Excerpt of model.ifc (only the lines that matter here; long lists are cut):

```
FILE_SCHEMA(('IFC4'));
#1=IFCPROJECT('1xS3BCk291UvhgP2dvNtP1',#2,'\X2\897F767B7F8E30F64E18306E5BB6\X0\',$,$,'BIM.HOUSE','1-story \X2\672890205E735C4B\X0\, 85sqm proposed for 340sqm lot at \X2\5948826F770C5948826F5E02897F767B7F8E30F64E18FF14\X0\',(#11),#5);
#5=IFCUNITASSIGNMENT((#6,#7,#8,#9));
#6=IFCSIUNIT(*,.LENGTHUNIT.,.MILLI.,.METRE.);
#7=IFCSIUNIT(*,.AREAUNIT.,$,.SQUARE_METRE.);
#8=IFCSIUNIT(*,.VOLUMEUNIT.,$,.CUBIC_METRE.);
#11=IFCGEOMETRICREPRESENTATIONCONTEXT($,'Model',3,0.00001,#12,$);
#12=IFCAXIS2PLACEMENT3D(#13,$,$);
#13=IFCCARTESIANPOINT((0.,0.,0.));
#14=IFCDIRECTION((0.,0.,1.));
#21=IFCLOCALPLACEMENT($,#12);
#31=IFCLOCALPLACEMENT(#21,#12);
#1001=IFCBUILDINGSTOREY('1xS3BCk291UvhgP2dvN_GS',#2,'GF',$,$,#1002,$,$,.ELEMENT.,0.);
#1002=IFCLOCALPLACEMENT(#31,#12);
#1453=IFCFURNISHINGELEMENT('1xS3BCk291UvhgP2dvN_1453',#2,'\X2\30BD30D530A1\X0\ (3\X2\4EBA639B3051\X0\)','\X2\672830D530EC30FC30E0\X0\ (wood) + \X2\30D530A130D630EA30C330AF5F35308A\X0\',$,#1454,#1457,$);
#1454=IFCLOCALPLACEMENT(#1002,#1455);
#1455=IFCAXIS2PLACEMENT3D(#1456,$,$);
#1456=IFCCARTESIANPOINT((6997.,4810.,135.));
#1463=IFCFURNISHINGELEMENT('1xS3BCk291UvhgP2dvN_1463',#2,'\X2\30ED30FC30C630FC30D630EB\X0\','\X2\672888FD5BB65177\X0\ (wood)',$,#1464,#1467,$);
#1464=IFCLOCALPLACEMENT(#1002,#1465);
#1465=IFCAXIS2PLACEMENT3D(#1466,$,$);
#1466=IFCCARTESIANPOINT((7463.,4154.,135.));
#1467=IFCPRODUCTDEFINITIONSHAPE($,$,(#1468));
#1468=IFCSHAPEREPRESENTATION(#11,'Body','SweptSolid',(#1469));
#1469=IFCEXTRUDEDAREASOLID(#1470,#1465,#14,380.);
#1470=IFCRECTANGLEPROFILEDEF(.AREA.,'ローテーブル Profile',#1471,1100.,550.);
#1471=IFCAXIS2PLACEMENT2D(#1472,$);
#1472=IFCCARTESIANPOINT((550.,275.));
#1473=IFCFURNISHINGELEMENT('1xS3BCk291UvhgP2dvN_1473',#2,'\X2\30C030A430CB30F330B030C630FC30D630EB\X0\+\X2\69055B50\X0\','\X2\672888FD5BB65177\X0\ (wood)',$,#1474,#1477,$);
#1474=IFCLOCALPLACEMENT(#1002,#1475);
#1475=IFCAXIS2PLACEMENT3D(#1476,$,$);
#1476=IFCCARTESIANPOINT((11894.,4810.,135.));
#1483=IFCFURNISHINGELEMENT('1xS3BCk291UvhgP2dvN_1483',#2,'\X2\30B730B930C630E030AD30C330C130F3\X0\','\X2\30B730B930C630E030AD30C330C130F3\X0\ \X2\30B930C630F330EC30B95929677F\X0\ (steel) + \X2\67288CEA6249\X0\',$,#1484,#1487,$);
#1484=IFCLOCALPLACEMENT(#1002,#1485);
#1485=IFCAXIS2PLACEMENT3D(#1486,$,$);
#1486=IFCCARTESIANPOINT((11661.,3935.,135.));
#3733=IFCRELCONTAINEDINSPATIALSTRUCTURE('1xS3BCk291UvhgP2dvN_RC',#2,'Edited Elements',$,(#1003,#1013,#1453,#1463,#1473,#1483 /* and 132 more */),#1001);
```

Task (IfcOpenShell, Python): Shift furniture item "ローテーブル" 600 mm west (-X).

```python
import ifcopenshell
import ifcopenshell.api.geometry
import ifcopenshell.util.placement

model = ifcopenshell.open("model.ifc")

item = model.by_id(1463)
matrix = ifcopenshell.util.placement.get_local_placement(item.ObjectPlacement)
matrix[0, 3] -= 600.0
ifcopenshell.api.geometry.edit_object_placement(model, product=item, matrix=matrix, is_si=False)

print(ifcopenshell.util.placement.get_local_placement(item.ObjectPlacement).round(3) + 0.0)

model.write("model-out.ifc")
```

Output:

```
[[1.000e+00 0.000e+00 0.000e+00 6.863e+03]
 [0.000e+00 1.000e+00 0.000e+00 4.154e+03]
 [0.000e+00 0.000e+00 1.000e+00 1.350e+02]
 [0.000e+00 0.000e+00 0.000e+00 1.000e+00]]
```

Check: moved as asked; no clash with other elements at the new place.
